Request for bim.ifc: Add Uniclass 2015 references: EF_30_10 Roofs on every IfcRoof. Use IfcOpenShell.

First a look at what the model holds.

```python
import ifcopenshell

model = ifcopenshell.open("bim.ifc")
print(model.schema)
print("classifications:", [c.Name for c in model.by_type("IfcClassification")])
for ifc_class in ("IfcDoor", "IfcRoof", "IfcStair", "IfcWall", "IfcWindow"):
    print(ifc_class, len(model.by_type(ifc_class)))
```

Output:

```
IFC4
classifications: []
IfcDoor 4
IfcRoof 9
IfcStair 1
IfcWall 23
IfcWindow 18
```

```python
import ifcopenshell
import ifcopenshell.api.classification

model = ifcopenshell.open("bim.ifc")

system = ifcopenshell.api.classification.add_classification(model, classification="Uniclass 2015")

codes = {
    "IfcRoof": ("EF_30_10", "Roofs"),
}
for ifc_class, (code, name) in codes.items():
    products = model.by_type(ifc_class)
    ifcopenshell.api.classification.add_reference(
        model, products=products, classification=system, identification=code, name=name
    )
    print(code, len(products))

model.write("bim_edited.ifc")
```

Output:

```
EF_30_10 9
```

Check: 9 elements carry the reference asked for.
